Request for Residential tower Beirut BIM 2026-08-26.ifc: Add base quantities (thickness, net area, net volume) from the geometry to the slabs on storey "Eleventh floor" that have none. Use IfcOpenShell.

First a look at what the model holds.

```python
import ifcopenshell
import ifcopenshell.util.element
import ifcopenshell.util.unit

model = ifcopenshell.open("Residential tower Beirut BIM 2026-08-26.ifc")
print(model.schema)
for unit_type in ("LENGTHUNIT", "AREAUNIT", "VOLUMEUNIT"):
    print(unit_type, ifcopenshell.util.unit.calculate_unit_scale(model, unit_type))
storey = next(s for s in model.by_type("IfcBuildingStorey") if s.Name == "Eleventh floor")
slabs = [e for e in ifcopenshell.util.element.get_decomposition(storey) if e.is_a("IfcSlab")]
for e in sorted(slabs, key=lambda e: e.id()):
    print(e.id(), e.is_a(), e.Name, list(ifcopenshell.util.element.get_psets(e, qtos_only=True)), sep=" | ")
```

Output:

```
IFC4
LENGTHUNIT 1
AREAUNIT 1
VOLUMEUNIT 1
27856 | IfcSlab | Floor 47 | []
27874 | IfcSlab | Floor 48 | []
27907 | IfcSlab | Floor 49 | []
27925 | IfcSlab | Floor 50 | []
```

```python
import ifcopenshell
import ifcopenshell.api.pset
import ifcopenshell.geom
import ifcopenshell.util.element
import ifcopenshell.util.shape
import ifcopenshell.util.unit

model = ifcopenshell.open("Residential tower Beirut BIM 2026-08-26.ifc")
unit_scale = ifcopenshell.util.unit.calculate_unit_scale(model)
area_scale = ifcopenshell.util.unit.calculate_unit_scale(model, "AREAUNIT")
volume_scale = ifcopenshell.util.unit.calculate_unit_scale(model, "VOLUMEUNIT")
settings = ifcopenshell.geom.settings()

storey = next(s for s in model.by_type("IfcBuildingStorey") if s.Name == "Eleventh floor")
slabs = [e for e in ifcopenshell.util.element.get_decomposition(storey) if e.is_a("IfcSlab")]

for e in sorted(slabs, key=lambda e: e.id()):
    if ifcopenshell.util.element.get_psets(e, qtos_only=True, should_inherit=False):
        continue
    # Geometry comes back in metres, in the element's own axes.
    shape = ifcopenshell.geom.create_shape(settings, e)
    values = {
        "Width": ifcopenshell.util.shape.get_z(shape.geometry) / unit_scale,
        "NetArea": ifcopenshell.util.shape.get_footprint_area(shape.geometry) / area_scale,
        "NetVolume": ifcopenshell.util.shape.get_volume(shape.geometry) / volume_scale,
    }
    qto = ifcopenshell.api.pset.add_qto(model, product=e, name="Qto_SlabBaseQuantities")
    ifcopenshell.api.pset.edit_qto(model, qto=qto, properties=values)
    print(e.id(), {k: round(v, 3) for k, v in values.items()})

model.write("Residential tower Beirut BIM 2026-08-26-out.ifc")
```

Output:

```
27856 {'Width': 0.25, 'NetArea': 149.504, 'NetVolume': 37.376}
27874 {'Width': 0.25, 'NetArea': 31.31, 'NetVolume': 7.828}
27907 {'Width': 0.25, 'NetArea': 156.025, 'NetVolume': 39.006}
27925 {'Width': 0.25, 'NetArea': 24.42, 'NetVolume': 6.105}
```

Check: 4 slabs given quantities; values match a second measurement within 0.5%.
